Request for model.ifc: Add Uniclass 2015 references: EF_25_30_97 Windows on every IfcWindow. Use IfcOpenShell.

First a look at what the model holds.

```python
import ifcopenshell

model = ifcopenshell.open("model.ifc")
print(model.schema)
print("classifications:", [c.Name for c in model.by_type("IfcClassification")])
for ifc_class in ("IfcDoor", "IfcRoof", "IfcStair", "IfcWall", "IfcWindow"):
    print(ifc_class, len(model.by_type(ifc_class)))
```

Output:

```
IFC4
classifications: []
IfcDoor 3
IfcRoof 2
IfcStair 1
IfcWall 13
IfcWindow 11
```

```python
import ifcopenshell
import ifcopenshell.api.classification

model = ifcopenshell.open("model.ifc")

system = ifcopenshell.api.classification.add_classification(model, classification="Uniclass 2015")

codes = {
    "IfcWindow": ("EF_25_30_97", "Windows"),
}
for ifc_class, (code, name) in codes.items():
    products = model.by_type(ifc_class)
    ifcopenshell.api.classification.add_reference(
        model, products=products, classification=system, identification=code, name=name
    )
    print(code, len(products))

model.write("model_updated.ifc")
```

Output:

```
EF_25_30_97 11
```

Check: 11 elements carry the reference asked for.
